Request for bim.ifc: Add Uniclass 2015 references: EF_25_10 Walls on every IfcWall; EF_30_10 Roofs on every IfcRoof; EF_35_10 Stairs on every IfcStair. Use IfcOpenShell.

First a look at what the model holds.

```python
import ifcopenshell

model = ifcopenshell.open("bim.ifc")
print(model.schema)
print("classifications:", [c.Name for c in model.by_type("IfcClassification")])
for ifc_class in ("IfcDoor", "IfcRoof", "IfcStair", "IfcWall", "IfcWindow"):
    print(ifc_class, len(model.by_type(ifc_class)))
```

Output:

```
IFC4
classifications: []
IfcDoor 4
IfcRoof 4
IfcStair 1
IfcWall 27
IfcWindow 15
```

```python
import ifcopenshell
import ifcopenshell.api.classification

model = ifcopenshell.open("bim.ifc")

system = ifcopenshell.api.classification.add_classification(model, classification="Uniclass 2015")

codes = {
    "IfcWall": ("EF_25_10", "Walls"),
    "IfcRoof": ("EF_30_10", "Roofs"),
    "IfcStair": ("EF_35_10", "Stairs"),
}
for ifc_class, (code, name) in codes.items():
    products = model.by_type(ifc_class)
    ifcopenshell.api.classification.add_reference(
        model, products=products, classification=system, identification=code, name=name
    )
    print(code, len(products))

model.write("bim_updated.ifc")
```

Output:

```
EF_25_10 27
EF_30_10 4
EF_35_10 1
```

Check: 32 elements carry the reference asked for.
